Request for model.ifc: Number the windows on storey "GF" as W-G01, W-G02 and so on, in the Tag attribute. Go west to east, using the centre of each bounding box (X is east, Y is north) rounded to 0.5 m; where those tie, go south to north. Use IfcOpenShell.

First a look at what the model holds.

```python
import ifcopenshell
import ifcopenshell.util.element
import ifcopenshell.util.placement

model = ifcopenshell.open("model.ifc")
print(model.schema)
storey = next(s for s in model.by_type("IfcBuildingStorey") if s.Name == "GF")
windows = [e for e in ifcopenshell.util.element.get_decomposition(storey) if e.is_a("IfcWindow")]
for e in sorted(windows, key=lambda e: e.id()):
    origin = ifcopenshell.util.placement.get_local_placement(e.ObjectPlacement)[:3, 3]
    print(e.id(), e.Tag, e.Name, origin.round(2) + 0.0, sep=" | ")
```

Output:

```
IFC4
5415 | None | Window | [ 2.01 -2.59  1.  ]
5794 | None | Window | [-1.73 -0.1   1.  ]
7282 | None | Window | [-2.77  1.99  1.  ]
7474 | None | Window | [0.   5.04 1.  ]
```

```python
import ifcopenshell
import ifcopenshell.geom
import ifcopenshell.util.element
import ifcopenshell.util.shape

model = ifcopenshell.open("model.ifc")
settings = ifcopenshell.geom.settings()
settings.set("use-world-coords", True)


def centre(element):
    shape = ifcopenshell.geom.create_shape(settings, element)
    return ifcopenshell.util.shape.get_bbox_centroid(shape.geometry)


storey = next(s for s in model.by_type("IfcBuildingStorey") if s.Name == "GF")
windows = [e for e in ifcopenshell.util.element.get_decomposition(storey) if e.is_a("IfcWindow")]

# Insertion points can sit at a corner or the storey origin, so sort by the geometry (in metres).
centres = {e: centre(e) for e in windows}
windows.sort(key=lambda e: (round(centres[e][0] / 0.5), centres[e][1]))

for i, e in enumerate(windows, start=1):
    number = f"W-G{i:02d}"
    e.Tag = number
    print(e.id(), number)

model.write("model-out.ifc")
```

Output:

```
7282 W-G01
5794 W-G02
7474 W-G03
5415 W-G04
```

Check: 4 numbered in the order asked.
